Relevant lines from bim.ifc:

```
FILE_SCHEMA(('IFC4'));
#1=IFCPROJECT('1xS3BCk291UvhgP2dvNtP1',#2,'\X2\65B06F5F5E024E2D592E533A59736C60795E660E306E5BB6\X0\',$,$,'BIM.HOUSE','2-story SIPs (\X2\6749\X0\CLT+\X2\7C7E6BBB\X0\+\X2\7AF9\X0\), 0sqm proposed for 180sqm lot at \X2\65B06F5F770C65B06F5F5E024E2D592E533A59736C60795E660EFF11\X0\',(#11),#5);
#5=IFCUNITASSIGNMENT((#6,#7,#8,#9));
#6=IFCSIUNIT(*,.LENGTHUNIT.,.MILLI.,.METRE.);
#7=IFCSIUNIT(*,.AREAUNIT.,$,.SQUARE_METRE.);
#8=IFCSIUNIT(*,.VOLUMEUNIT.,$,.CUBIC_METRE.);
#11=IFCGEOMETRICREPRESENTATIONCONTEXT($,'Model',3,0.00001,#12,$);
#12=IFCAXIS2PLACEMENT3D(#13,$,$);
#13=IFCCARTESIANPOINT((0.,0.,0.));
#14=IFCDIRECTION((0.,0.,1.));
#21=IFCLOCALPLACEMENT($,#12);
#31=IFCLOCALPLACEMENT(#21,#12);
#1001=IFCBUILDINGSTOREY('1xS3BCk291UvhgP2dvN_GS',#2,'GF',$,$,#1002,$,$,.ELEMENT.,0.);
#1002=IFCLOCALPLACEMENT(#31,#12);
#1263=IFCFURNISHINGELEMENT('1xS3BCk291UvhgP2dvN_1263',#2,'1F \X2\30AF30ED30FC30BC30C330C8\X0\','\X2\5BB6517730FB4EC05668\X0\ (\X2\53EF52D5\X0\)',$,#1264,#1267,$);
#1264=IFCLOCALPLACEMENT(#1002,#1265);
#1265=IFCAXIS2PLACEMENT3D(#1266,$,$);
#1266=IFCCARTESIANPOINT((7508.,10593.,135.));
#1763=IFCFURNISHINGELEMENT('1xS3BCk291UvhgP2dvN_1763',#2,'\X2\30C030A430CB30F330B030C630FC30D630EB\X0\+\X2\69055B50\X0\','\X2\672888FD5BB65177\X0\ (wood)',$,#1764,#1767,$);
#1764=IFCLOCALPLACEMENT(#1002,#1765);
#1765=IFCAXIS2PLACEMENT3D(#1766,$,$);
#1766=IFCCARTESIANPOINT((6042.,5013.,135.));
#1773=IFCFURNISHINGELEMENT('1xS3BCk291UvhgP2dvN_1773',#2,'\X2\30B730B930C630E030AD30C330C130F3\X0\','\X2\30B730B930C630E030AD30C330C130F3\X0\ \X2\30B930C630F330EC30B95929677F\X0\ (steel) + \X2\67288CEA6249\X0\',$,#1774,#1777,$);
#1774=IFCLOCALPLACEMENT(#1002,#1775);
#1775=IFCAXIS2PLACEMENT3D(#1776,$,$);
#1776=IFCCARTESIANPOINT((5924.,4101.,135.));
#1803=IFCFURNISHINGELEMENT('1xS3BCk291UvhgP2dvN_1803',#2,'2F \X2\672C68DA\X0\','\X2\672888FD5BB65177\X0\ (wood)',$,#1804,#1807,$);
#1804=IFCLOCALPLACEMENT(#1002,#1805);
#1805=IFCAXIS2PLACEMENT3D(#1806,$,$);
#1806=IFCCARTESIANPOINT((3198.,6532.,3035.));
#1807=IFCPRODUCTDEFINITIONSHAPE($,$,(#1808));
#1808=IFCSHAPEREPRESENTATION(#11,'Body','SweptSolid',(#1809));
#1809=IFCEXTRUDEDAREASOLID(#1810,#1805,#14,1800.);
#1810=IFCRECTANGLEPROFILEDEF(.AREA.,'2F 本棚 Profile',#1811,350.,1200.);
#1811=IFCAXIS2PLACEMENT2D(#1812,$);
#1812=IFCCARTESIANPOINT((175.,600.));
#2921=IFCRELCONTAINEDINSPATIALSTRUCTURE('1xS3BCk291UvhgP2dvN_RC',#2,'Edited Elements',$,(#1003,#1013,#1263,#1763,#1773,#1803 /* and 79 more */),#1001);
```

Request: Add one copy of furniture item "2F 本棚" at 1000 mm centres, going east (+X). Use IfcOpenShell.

```python
import numpy as np
import ifcopenshell
import ifcopenshell.api.geometry
import ifcopenshell.api.root
import ifcopenshell.util.element
import ifcopenshell.util.placement

model = ifcopenshell.open("bim.ifc")


def reuse_history(source, copy):
    """copy_class also copies each property set's owner history, people and application; keep the originals."""
    for rel in copy.IsDefinedBy:
        if rel.is_a("IfcRelDefinesByProperties") and (history := rel.RelatingPropertyDefinition.OwnerHistory):
            rel.RelatingPropertyDefinition.OwnerHistory = source.OwnerHistory
            ifcopenshell.util.element.remove_deep2(model, history)


source = model.by_id(1803)
base = ifcopenshell.util.placement.get_local_placement(source.ObjectPlacement)
step = np.array([1.0, 0.0, 0.0]) * 1000.0

for i in range(1, 2):
    copy = ifcopenshell.api.root.copy_class(model, product=source)
    copy.Representation = ifcopenshell.util.element.copy_deep(
        model, source.Representation, exclude=["IfcGeometricRepresentationContext", "IfcRepresentationMap"]
    )
    reuse_history(source, copy)
    matrix = base.copy()
    matrix[:3, 3] += i * step
    print("added at", matrix[:3, 3].round(3) + 0.0)
    ifcopenshell.api.geometry.edit_object_placement(model, product=copy, matrix=matrix, is_si=False)

model.write("bim-out.ifc")
```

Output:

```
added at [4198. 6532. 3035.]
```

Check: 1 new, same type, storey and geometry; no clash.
